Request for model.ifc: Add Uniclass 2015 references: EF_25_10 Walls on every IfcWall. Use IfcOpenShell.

First a look at what the model holds.

```python
import ifcopenshell

model = ifcopenshell.open("model.ifc")
print(model.schema)
print("classifications:", [c.Name for c in model.by_type("IfcClassification")])
for ifc_class in ("IfcDoor", "IfcRoof", "IfcStair", "IfcWall", "IfcWindow"):
    print(ifc_class, len(model.by_type(ifc_class)))
```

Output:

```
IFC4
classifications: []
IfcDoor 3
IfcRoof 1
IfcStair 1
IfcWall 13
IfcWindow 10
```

```python
import ifcopenshell
import ifcopenshell.api.classification

model = ifcopenshell.open("model.ifc")

system = ifcopenshell.api.classification.add_classification(model, classification="Uniclass 2015")

codes = {
    "IfcWall": ("EF_25_10", "Walls"),
}
for ifc_class, (code, name) in codes.items():
    products = model.by_type(ifc_class)
    ifcopenshell.api.classification.add_reference(
        model, products=products, classification=system, identification=code, name=name
    )
    print(code, len(products))

model.write("model_rev.ifc")
```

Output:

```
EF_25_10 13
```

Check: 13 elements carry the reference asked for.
